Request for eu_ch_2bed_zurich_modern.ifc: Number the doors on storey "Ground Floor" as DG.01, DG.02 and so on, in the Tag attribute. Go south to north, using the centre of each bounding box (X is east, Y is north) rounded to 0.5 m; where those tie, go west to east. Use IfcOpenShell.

First a look at what the model holds.

```python
import ifcopenshell
import ifcopenshell.util.element
import ifcopenshell.util.placement

model = ifcopenshell.open("eu_ch_2bed_zurich_modern.ifc")
print(model.schema)
storey = next(s for s in model.by_type("IfcBuildingStorey") if s.Name == "Ground Floor")
doors = [e for e in ifcopenshell.util.element.get_decomposition(storey) if e.is_a("IfcDoor")]
for e in sorted(doors, key=lambda e: e.id()):
    origin = ifcopenshell.util.placement.get_local_placement(e.ObjectPlacement)[:3, 3]
    print(e.id(), e.Tag, e.Name, origin.round(2) + 0.0, sep=" | ")
```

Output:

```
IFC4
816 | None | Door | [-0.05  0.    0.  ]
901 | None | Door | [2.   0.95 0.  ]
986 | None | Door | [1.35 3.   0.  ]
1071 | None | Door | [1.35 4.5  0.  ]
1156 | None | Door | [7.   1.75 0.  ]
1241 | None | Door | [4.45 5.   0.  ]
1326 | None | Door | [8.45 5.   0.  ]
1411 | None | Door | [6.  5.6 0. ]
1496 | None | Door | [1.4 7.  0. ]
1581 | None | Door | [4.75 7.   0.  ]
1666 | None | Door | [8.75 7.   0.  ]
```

```python
import ifcopenshell
import ifcopenshell.geom
import ifcopenshell.util.element
import ifcopenshell.util.shape

model = ifcopenshell.open("eu_ch_2bed_zurich_modern.ifc")
settings = ifcopenshell.geom.settings()
settings.set("use-world-coords", True)


def centre(element):
    shape = ifcopenshell.geom.create_shape(settings, element)
    return ifcopenshell.util.shape.get_bbox_centroid(shape.geometry)


storey = next(s for s in model.by_type("IfcBuildingStorey") if s.Name == "Ground Floor")
doors = [e for e in ifcopenshell.util.element.get_decomposition(storey) if e.is_a("IfcDoor")]

# Insertion points can sit at a corner or the storey origin, so sort by the geometry (in metres).
centres = {e: centre(e) for e in doors}
doors.sort(key=lambda e: (round(centres[e][1] / 0.5), centres[e][0]))

for i, e in enumerate(doors, start=1):
    number = f"DG.{i:02d}"
    e.Tag = number
    print(e.id(), number)

model.write("eu_ch_2bed_zurich_modern-out.ifc")
```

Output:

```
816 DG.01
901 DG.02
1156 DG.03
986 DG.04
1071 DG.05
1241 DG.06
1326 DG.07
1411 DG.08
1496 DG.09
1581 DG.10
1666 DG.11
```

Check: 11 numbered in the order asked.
